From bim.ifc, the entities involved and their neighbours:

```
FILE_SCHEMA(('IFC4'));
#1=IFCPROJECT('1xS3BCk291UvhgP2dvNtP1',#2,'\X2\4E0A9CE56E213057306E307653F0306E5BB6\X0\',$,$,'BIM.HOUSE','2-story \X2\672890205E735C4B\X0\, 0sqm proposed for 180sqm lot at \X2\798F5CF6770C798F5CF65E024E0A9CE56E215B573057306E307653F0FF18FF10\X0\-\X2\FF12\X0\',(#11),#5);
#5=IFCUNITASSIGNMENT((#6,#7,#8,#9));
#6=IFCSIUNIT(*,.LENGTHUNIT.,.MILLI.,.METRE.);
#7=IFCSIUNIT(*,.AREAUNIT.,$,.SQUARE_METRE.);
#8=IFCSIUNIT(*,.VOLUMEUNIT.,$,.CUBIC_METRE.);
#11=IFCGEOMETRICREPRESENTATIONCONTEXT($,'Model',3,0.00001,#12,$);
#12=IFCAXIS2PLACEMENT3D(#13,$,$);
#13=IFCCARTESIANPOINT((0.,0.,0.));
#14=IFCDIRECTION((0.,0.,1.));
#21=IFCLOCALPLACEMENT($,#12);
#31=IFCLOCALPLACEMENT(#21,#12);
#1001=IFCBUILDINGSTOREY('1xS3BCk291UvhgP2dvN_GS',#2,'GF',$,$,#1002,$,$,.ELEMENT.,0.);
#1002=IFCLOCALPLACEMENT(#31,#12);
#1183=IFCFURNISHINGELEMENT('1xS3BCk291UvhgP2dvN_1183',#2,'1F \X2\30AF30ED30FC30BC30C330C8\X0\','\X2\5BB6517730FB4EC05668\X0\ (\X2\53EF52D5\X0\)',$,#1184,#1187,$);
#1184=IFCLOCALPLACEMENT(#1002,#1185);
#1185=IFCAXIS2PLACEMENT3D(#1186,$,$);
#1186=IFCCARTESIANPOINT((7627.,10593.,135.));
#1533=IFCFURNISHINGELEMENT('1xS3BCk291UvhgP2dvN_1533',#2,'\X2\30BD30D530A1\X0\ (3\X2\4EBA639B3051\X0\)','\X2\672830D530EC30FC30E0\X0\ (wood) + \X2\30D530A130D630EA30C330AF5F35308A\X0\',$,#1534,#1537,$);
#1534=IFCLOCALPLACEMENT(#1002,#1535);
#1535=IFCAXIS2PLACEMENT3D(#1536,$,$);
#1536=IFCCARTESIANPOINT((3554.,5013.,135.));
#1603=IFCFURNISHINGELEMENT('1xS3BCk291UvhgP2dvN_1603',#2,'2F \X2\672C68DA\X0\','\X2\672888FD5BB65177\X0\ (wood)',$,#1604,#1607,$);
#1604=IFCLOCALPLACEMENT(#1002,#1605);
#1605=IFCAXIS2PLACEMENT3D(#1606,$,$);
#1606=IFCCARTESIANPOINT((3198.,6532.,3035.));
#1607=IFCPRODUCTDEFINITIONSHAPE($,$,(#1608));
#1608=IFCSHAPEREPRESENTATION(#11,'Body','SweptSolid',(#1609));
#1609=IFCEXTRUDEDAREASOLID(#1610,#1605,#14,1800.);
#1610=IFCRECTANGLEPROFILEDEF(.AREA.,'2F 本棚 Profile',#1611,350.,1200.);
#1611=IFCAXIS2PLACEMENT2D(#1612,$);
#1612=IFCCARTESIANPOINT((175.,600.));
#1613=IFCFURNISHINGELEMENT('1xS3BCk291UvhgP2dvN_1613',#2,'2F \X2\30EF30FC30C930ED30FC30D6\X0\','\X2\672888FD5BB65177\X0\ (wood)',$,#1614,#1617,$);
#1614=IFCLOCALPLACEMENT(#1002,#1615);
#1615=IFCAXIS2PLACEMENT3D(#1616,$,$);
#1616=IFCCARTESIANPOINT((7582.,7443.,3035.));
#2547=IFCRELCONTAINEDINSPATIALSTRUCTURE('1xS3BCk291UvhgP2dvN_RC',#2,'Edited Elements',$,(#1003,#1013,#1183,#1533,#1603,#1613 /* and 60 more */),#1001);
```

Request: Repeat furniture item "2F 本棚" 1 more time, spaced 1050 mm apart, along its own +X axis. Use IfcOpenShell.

```python
import ifcopenshell
import ifcopenshell.api.geometry
import ifcopenshell.api.root
import ifcopenshell.util.element
import ifcopenshell.util.placement
import ifcopenshell.util.unit

model = ifcopenshell.open("bim.ifc")
unit_scale = ifcopenshell.util.unit.calculate_unit_scale(model)


def reuse_history(source, copy):
    """copy_class also copies each property set's owner history, people and application; keep the originals."""
    for rel in copy.IsDefinedBy:
        if rel.is_a("IfcRelDefinesByProperties") and (history := rel.RelatingPropertyDefinition.OwnerHistory):
            rel.RelatingPropertyDefinition.OwnerHistory = source.OwnerHistory
            ifcopenshell.util.element.remove_deep2(model, history)


source = model.by_id(1603)
base = ifcopenshell.util.placement.get_local_placement(source.ObjectPlacement)
step = base[:3, 0] * 1.05 / unit_scale

for i in range(1, 2):
    copy = ifcopenshell.api.root.copy_class(model, product=source)
    copy.Representation = ifcopenshell.util.element.copy_deep(
        model, source.Representation, exclude=["IfcGeometricRepresentationContext", "IfcRepresentationMap"]
    )
    reuse_history(source, copy)
    matrix = base.copy()
    matrix[:3, 3] += i * step
    print("added at", matrix[:3, 3].round(3) + 0.0)
    ifcopenshell.api.geometry.edit_object_placement(model, product=copy, matrix=matrix, is_si=False)

model.write("bim-out.ifc")
```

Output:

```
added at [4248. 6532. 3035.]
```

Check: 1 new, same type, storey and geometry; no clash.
